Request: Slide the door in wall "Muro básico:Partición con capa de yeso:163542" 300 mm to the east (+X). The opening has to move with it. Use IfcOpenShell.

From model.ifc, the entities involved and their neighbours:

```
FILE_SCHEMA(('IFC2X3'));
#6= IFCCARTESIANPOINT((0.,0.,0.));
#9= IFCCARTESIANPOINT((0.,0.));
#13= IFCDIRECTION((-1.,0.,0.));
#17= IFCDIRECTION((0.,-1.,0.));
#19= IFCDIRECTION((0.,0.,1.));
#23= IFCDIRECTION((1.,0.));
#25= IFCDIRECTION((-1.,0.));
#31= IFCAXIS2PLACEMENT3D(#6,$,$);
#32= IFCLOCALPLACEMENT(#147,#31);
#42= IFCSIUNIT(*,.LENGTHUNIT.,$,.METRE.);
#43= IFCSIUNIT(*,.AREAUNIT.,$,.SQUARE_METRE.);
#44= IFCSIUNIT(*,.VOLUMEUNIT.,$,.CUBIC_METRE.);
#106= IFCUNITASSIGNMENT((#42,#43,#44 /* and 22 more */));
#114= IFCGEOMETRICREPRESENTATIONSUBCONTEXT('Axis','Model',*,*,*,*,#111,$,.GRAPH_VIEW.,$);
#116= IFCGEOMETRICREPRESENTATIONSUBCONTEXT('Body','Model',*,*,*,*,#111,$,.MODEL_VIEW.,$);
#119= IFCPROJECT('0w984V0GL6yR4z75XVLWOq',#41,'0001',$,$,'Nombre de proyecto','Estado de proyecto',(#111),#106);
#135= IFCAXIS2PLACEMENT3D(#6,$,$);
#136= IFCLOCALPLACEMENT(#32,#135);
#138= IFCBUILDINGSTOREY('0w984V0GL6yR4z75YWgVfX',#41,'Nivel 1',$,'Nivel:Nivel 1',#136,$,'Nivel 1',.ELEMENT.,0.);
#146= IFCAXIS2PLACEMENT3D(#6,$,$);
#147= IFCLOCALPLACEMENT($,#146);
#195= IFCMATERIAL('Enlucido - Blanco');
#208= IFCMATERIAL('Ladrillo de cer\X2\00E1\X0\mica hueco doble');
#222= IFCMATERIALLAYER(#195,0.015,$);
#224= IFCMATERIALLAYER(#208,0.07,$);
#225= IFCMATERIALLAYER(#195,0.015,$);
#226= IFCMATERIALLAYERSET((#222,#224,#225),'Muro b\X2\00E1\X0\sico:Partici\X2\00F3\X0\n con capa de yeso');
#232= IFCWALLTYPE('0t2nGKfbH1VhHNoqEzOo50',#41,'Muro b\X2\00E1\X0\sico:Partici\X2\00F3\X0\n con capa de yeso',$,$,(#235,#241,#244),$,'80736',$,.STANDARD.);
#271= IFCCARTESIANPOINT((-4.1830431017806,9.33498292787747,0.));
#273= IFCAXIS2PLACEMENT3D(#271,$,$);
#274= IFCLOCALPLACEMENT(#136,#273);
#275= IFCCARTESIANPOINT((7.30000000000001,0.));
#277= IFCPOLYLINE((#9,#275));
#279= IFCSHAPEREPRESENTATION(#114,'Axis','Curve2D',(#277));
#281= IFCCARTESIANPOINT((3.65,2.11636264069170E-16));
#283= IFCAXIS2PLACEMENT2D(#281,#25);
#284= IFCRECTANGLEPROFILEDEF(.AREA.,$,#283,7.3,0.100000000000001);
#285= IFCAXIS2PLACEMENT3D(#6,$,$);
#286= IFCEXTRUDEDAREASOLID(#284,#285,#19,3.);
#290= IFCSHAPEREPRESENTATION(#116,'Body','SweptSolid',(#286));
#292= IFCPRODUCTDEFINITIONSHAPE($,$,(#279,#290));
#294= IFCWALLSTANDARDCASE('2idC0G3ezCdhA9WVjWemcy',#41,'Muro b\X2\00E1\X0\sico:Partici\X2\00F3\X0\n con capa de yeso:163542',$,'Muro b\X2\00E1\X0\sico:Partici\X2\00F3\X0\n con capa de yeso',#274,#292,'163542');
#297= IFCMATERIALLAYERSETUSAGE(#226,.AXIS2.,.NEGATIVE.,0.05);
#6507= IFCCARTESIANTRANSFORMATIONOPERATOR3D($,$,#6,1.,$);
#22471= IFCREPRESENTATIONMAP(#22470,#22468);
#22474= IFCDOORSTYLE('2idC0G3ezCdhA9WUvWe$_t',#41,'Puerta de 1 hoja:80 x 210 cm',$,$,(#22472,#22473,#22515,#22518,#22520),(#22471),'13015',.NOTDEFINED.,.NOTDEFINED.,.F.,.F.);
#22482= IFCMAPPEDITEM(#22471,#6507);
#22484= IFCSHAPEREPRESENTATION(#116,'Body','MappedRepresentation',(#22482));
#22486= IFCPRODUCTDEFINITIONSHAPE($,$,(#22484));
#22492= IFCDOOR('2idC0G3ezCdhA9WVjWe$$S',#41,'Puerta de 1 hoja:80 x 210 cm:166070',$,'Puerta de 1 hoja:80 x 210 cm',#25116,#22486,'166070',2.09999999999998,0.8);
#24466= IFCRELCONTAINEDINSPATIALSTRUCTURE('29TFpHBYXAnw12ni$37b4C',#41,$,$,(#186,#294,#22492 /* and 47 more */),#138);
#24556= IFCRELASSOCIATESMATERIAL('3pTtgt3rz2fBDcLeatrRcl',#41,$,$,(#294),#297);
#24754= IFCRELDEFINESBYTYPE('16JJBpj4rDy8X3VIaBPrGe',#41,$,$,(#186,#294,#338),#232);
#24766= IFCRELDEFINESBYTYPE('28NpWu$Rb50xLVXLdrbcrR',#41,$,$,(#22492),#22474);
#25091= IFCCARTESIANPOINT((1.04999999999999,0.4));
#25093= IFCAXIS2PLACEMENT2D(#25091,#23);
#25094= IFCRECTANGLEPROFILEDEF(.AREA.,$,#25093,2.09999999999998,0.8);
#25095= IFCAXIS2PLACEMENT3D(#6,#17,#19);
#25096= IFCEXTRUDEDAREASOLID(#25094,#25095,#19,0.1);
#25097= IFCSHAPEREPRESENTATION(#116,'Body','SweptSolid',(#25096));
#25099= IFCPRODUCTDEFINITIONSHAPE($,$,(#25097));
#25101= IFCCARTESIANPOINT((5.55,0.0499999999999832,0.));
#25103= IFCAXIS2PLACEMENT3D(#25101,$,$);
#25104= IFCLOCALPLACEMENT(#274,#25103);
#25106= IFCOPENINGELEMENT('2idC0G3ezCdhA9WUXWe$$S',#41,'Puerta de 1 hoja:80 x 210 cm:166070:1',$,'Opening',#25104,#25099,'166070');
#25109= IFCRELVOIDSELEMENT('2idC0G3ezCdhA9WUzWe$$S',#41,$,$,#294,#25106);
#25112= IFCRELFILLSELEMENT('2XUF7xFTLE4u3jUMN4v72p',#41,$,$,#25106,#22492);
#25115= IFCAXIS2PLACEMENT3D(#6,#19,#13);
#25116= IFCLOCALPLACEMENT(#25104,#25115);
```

```python
import ifcopenshell
import ifcopenshell.api.geometry
import ifcopenshell.util.placement

model = ifcopenshell.open("model.ifc")

door = model.by_guid("2idC0G3ezCdhA9WVjWe$$S")
opening = door.FillsVoids[0].RelatingOpeningElement
wall = opening.VoidsElements[0].RelatingBuildingElement

wall_matrix = ifcopenshell.util.placement.get_local_placement(wall.ObjectPlacement)
shift = wall_matrix[:3, 0] * 0.3
before = ifcopenshell.util.placement.get_local_placement(door.ObjectPlacement)[:3, 3].copy()

# The door is placed relative to its opening, so it follows when the opening moves.
matrix = ifcopenshell.util.placement.get_local_placement(opening.ObjectPlacement)
matrix[:3, 3] += shift
ifcopenshell.api.geometry.edit_object_placement(
    model, product=opening, matrix=matrix, is_si=False, should_transform_children=True
)

after = ifcopenshell.util.placement.get_local_placement(door.ObjectPlacement)[:3, 3]
print("door moved by", (after - before).round(3) + 0.0)

model.write("model-out.ifc")
```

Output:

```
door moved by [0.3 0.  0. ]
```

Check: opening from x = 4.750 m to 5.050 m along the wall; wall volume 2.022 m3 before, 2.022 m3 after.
